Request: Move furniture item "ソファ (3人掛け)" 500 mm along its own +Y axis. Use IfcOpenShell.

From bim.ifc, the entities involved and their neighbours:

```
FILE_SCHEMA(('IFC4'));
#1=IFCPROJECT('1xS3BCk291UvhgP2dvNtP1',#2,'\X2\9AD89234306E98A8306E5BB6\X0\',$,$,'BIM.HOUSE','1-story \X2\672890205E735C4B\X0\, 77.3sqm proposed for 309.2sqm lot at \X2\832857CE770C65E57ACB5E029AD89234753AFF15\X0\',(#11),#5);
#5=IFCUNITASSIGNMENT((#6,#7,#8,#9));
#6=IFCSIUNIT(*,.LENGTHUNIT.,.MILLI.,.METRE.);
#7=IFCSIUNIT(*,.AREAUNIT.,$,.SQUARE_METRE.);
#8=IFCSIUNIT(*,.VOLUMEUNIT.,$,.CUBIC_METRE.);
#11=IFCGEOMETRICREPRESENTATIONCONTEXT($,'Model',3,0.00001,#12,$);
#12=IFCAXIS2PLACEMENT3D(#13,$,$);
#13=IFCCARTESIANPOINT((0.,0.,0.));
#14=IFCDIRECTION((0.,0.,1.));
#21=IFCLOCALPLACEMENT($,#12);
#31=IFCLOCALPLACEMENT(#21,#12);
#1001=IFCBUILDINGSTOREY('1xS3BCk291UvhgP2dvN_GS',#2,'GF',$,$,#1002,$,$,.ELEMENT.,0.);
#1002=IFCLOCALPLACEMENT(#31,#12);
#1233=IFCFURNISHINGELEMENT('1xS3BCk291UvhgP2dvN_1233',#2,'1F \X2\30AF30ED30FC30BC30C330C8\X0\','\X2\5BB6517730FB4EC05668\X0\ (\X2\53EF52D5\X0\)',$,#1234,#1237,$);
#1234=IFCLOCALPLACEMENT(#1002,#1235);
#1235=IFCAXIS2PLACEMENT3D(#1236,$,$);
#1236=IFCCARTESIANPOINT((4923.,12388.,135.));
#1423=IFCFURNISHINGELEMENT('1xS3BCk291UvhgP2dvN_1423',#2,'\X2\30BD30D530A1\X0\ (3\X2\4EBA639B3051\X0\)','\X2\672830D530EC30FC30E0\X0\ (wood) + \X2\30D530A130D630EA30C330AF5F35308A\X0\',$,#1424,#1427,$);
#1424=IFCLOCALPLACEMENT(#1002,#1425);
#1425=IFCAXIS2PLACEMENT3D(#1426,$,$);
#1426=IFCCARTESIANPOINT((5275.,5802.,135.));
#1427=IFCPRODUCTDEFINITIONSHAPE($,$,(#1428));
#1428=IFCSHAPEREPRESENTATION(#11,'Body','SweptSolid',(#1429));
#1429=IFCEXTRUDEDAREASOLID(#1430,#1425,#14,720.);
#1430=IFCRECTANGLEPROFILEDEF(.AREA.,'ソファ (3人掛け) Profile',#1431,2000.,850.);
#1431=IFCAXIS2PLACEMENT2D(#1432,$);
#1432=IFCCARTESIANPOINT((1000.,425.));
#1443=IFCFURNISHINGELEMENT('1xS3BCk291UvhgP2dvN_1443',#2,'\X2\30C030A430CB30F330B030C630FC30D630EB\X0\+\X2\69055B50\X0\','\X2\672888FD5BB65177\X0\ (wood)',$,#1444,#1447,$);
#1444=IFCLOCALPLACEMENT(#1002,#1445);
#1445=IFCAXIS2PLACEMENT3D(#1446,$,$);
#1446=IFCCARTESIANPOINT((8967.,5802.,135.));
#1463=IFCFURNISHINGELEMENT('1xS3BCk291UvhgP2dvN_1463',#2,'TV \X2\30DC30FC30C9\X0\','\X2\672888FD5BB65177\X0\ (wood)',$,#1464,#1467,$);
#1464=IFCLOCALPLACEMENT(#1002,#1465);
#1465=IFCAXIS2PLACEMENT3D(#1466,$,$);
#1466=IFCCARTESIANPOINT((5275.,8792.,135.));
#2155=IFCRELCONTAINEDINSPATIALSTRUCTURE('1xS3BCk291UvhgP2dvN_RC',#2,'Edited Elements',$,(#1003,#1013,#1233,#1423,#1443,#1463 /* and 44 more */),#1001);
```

```python
import ifcopenshell
import ifcopenshell.api.geometry
import ifcopenshell.util.placement
import ifcopenshell.util.unit

model = ifcopenshell.open("bim.ifc")
unit_scale = ifcopenshell.util.unit.calculate_unit_scale(model)

item = model.by_guid("1xS3BCk291UvhgP2dvN_1423")
matrix = ifcopenshell.util.placement.get_local_placement(item.ObjectPlacement)
matrix[:3, 3] += matrix[:3, 1] * 0.5 / unit_scale
ifcopenshell.api.geometry.edit_object_placement(model, product=item, matrix=matrix, is_si=False)

print(ifcopenshell.util.placement.get_local_placement(item.ObjectPlacement).round(3) + 0.0)

model.write("bim_updated.ifc")
```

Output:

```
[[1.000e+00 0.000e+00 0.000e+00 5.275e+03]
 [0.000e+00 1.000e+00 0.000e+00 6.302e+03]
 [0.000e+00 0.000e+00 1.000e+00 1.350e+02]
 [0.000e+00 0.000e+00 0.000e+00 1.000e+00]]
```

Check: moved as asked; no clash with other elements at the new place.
